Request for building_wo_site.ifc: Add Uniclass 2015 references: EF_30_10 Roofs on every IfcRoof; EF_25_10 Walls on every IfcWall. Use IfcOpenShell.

First a look at what the model holds.

```python
import ifcopenshell

model = ifcopenshell.open("building_wo_site.ifc")
print(model.schema)
print("classifications:", [c.Name for c in model.by_type("IfcClassification")])
for ifc_class in ("IfcDoor", "IfcRoof", "IfcStair", "IfcWall", "IfcWindow"):
    print(ifc_class, len(model.by_type(ifc_class)))
```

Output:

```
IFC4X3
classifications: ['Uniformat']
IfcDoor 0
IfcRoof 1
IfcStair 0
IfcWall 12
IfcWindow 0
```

```python
import ifcopenshell
import ifcopenshell.api.classification

model = ifcopenshell.open("building_wo_site.ifc")

system = ifcopenshell.api.classification.add_classification(model, classification="Uniclass 2015")

codes = {
    "IfcRoof": ("EF_30_10", "Roofs"),
    "IfcWall": ("EF_25_10", "Walls"),
}
for ifc_class, (code, name) in codes.items():
    products = model.by_type(ifc_class)
    ifcopenshell.api.classification.add_reference(
        model, products=products, classification=system, identification=code, name=name
    )
    print(code, len(products))

model.write("building_wo_site_edited.ifc")
```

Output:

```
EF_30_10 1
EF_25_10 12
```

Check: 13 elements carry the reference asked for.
